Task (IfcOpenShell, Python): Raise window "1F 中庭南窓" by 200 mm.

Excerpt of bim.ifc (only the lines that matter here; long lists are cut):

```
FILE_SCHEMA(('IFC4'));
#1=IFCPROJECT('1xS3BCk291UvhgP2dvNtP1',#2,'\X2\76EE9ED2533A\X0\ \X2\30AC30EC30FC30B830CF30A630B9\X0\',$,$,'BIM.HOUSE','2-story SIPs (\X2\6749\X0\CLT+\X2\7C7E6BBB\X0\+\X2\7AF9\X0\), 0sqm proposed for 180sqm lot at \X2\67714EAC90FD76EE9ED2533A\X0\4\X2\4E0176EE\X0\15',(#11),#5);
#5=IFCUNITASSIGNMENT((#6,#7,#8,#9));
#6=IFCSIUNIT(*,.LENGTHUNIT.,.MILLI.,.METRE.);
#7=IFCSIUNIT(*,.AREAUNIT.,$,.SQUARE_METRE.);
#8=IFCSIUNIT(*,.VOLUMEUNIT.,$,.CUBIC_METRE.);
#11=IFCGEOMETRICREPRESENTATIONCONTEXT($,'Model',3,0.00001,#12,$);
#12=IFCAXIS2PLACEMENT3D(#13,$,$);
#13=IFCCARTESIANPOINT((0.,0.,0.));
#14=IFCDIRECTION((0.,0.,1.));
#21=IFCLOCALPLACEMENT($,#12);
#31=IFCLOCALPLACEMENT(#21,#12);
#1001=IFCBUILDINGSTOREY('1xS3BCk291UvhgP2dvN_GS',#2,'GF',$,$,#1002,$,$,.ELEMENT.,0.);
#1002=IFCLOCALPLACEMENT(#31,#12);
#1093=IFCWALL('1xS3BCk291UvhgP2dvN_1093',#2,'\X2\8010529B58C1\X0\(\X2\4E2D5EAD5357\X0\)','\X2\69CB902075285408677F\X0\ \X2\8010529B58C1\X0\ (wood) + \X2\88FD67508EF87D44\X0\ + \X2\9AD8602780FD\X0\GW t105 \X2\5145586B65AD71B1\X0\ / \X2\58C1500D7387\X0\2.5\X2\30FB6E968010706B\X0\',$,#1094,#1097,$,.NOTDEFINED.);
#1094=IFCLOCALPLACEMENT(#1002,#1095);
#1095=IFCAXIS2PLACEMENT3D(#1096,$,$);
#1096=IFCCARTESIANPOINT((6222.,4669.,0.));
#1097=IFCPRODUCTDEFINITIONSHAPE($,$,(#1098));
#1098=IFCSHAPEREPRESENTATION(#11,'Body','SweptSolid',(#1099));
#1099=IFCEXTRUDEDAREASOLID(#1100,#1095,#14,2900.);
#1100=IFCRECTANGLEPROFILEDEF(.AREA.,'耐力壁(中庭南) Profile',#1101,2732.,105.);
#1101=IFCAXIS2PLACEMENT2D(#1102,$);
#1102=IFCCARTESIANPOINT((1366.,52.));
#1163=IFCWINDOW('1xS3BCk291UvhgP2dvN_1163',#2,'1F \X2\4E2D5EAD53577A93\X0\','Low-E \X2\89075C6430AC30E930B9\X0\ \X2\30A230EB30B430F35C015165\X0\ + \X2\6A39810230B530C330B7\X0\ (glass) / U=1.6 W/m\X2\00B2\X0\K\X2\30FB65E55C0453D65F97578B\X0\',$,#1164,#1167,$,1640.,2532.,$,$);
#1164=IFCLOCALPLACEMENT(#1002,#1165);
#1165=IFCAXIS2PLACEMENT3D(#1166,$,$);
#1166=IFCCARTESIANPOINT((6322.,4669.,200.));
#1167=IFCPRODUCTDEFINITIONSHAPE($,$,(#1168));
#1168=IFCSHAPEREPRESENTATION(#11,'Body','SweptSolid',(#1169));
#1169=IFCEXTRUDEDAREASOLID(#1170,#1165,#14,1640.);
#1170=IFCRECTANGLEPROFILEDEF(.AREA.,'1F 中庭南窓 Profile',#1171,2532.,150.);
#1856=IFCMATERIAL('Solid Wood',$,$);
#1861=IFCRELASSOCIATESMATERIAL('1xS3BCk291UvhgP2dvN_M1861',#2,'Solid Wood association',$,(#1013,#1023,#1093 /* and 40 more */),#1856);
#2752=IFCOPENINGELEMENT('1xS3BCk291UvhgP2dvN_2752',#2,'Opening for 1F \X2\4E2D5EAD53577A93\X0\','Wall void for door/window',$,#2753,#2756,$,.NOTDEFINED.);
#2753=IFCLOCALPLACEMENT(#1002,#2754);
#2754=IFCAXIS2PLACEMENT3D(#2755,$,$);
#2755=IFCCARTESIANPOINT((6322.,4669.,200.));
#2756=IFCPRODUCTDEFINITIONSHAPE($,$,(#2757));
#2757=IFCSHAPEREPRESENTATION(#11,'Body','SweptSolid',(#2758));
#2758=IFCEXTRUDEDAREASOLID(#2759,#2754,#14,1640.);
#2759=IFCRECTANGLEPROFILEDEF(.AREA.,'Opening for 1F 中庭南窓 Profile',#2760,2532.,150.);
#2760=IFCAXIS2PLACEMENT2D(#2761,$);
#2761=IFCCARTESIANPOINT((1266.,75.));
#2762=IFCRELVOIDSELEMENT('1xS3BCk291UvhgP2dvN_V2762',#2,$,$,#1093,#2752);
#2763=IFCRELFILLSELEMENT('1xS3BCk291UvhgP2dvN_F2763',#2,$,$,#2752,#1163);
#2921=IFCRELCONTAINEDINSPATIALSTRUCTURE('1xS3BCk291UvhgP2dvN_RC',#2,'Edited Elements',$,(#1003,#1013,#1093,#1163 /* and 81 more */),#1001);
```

```python
import numpy as np
import ifcopenshell
import ifcopenshell.api.geometry
import ifcopenshell.util.placement
import ifcopenshell.util.unit

model = ifcopenshell.open("bim.ifc")
unit_scale = ifcopenshell.util.unit.calculate_unit_scale(model)

window = model.by_id(1163)
opening = window.FillsVoids[0].RelatingOpeningElement
dz = 200.0

shift = np.array([0.0, 0.0, dz])
# The window is not placed relative to its opening, so move both.
for product in (opening, window):
    matrix = ifcopenshell.util.placement.get_local_placement(product.ObjectPlacement)
    matrix[:3, 3] += shift
    ifcopenshell.api.geometry.edit_object_placement(model, product=product, matrix=matrix, is_si=False)

print(f"moved by {dz * unit_scale:+.3f} m")

model.write("bim_edited.ifc")
```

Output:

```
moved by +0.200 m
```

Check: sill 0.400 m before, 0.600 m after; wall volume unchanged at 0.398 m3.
